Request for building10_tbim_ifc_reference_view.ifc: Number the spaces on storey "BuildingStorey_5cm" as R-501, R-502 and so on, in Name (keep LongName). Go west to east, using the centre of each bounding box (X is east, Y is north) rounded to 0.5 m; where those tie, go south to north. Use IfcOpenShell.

First a look at what the model holds.

```python
import ifcopenshell
import ifcopenshell.util.element
import ifcopenshell.util.placement

model = ifcopenshell.open("building10_tbim_ifc_reference_view.ifc")
print(model.schema)
storey = next(s for s in model.by_type("IfcBuildingStorey") if s.Name == "BuildingStorey_5cm")
spaces = [e for e in ifcopenshell.util.element.get_decomposition(storey) if e.is_a("IfcSpace")]
for e in sorted(spaces, key=lambda e: e.id()):
    origin = ifcopenshell.util.placement.get_local_placement(e.ObjectPlacement)[:3, 3]
    print(e.id(), e.Name, e.LongName, origin.round(2) + 0.0, sep=" | ")
```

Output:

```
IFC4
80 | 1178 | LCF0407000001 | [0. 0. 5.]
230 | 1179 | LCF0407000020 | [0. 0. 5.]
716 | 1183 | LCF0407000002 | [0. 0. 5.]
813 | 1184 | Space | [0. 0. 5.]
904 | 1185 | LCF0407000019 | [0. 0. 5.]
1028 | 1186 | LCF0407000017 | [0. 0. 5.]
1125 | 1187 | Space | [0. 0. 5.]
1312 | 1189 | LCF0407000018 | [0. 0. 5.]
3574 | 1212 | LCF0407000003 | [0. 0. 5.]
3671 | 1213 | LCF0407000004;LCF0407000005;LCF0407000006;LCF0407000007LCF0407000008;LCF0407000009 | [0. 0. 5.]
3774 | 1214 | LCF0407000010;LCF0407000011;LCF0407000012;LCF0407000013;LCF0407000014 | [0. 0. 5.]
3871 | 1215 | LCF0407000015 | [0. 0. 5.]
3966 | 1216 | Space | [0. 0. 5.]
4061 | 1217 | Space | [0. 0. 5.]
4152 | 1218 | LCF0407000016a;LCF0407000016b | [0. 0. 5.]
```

```python
import ifcopenshell
import ifcopenshell.geom
import ifcopenshell.util.element
import ifcopenshell.util.shape

model = ifcopenshell.open("building10_tbim_ifc_reference_view.ifc")
settings = ifcopenshell.geom.settings()
settings.set("use-world-coords", True)


def centre(element):
    shape = ifcopenshell.geom.create_shape(settings, element)
    return ifcopenshell.util.shape.get_bbox_centroid(shape.geometry)


storey = next(s for s in model.by_type("IfcBuildingStorey") if s.Name == "BuildingStorey_5cm")
spaces = [e for e in ifcopenshell.util.element.get_decomposition(storey) if e.is_a("IfcSpace")]

# Insertion points can sit at a corner or the storey origin, so sort by the geometry (in metres).
centres = {e: centre(e) for e in spaces}
spaces.sort(key=lambda e: (round(centres[e][0] / 0.5), centres[e][1]))

for i, e in enumerate(spaces, start=1):
    number = f"R-5{i:02d}"
    e.Name = number
    print(e.id(), number)

model.write("building10_tbim_ifc_reference_view_rev.ifc")
```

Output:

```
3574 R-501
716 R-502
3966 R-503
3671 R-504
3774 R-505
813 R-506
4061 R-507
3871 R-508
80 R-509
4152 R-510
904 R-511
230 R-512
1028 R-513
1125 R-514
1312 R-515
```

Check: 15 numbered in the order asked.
